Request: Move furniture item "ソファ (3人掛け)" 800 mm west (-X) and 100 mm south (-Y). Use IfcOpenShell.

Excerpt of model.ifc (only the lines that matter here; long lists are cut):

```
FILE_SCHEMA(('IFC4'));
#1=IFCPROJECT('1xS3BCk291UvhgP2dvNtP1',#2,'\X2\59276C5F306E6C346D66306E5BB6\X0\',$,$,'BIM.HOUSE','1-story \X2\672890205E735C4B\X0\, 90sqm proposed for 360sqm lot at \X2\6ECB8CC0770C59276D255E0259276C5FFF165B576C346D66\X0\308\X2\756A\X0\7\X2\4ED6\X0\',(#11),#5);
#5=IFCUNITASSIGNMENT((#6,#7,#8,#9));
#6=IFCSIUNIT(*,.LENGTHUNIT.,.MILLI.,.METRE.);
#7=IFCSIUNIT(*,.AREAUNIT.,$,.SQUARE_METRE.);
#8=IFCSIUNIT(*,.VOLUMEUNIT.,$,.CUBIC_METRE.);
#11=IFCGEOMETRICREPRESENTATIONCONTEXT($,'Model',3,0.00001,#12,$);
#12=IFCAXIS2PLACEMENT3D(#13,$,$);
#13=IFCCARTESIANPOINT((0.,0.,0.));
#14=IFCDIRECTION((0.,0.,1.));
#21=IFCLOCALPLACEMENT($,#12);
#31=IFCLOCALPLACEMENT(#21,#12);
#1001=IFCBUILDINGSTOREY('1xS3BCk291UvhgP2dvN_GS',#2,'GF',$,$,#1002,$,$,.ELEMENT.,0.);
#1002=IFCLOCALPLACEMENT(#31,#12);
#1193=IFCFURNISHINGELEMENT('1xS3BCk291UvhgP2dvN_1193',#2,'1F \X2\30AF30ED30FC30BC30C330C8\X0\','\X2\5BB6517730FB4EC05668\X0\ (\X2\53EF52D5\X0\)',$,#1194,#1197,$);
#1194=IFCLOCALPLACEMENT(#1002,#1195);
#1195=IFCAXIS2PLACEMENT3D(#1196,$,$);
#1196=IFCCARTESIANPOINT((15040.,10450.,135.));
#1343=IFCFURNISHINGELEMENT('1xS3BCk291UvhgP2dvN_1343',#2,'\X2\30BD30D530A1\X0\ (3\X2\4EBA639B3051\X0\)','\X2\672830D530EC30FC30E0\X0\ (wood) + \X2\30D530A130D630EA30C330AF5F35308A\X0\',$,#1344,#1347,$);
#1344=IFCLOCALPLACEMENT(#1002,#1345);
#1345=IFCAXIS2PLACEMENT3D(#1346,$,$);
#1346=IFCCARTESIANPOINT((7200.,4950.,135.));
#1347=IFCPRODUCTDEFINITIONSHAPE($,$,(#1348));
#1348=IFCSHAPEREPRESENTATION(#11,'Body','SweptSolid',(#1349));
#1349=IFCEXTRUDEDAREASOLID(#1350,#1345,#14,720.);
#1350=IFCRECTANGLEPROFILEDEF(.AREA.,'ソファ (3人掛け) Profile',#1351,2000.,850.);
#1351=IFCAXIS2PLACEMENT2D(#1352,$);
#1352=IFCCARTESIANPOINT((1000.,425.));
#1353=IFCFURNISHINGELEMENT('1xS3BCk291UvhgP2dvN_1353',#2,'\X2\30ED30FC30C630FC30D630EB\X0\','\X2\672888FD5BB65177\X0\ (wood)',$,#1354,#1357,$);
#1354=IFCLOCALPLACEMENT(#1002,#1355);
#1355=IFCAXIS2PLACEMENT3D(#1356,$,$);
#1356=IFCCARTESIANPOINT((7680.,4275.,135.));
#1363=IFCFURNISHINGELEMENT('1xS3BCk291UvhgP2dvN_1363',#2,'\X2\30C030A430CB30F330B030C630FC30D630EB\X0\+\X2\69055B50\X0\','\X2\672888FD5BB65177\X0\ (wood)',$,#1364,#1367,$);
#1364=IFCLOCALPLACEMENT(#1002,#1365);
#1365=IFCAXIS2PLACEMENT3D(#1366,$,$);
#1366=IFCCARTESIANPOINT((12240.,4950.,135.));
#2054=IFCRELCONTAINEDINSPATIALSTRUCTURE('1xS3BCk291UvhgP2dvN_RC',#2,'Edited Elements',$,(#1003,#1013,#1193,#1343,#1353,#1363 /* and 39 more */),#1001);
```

```python
import ifcopenshell
import ifcopenshell.api.geometry
import ifcopenshell.util.placement

model = ifcopenshell.open("model.ifc")

item = model.by_guid("1xS3BCk291UvhgP2dvN_1343")
matrix = ifcopenshell.util.placement.get_local_placement(item.ObjectPlacement)
matrix[0, 3] -= 800.0
matrix[1, 3] -= 100.0
ifcopenshell.api.geometry.edit_object_placement(model, product=item, matrix=matrix, is_si=False)

print(ifcopenshell.util.placement.get_local_placement(item.ObjectPlacement).round(3) + 0.0)

model.write("model_updated.ifc")
```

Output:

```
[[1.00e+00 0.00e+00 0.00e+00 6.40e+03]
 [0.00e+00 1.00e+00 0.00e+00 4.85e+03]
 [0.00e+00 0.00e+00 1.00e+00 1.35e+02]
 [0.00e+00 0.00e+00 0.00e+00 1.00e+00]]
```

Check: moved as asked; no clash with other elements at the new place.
